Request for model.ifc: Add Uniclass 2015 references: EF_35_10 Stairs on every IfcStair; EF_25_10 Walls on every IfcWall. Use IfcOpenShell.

First a look at what the model holds.

```python
import ifcopenshell

model = ifcopenshell.open("model.ifc")
print(model.schema)
print("classifications:", [c.Name for c in model.by_type("IfcClassification")])
for ifc_class in ("IfcDoor", "IfcRoof", "IfcStair", "IfcWall", "IfcWindow"):
    print(ifc_class, len(model.by_type(ifc_class)))
```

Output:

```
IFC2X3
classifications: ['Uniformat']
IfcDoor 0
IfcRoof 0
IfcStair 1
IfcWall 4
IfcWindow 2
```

```python
import ifcopenshell
import ifcopenshell.api.classification

model = ifcopenshell.open("model.ifc")

# IFC2X3 requires Source and Edition and has no link from the project to the system.
system = model.create_entity("IfcClassification", Source="NBS", Edition="2015", Name="Uniclass 2015")

codes = {
    "IfcStair": ("EF_35_10", "Stairs"),
    "IfcWall": ("EF_25_10", "Walls"),
}
for ifc_class, (code, name) in codes.items():
    products = model.by_type(ifc_class)
    ifcopenshell.api.classification.add_reference(
        model, products=products, classification=system, identification=code, name=name
    )
    print(code, len(products))

model.write("model_updated.ifc")
```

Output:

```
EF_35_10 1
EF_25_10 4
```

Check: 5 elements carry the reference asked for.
